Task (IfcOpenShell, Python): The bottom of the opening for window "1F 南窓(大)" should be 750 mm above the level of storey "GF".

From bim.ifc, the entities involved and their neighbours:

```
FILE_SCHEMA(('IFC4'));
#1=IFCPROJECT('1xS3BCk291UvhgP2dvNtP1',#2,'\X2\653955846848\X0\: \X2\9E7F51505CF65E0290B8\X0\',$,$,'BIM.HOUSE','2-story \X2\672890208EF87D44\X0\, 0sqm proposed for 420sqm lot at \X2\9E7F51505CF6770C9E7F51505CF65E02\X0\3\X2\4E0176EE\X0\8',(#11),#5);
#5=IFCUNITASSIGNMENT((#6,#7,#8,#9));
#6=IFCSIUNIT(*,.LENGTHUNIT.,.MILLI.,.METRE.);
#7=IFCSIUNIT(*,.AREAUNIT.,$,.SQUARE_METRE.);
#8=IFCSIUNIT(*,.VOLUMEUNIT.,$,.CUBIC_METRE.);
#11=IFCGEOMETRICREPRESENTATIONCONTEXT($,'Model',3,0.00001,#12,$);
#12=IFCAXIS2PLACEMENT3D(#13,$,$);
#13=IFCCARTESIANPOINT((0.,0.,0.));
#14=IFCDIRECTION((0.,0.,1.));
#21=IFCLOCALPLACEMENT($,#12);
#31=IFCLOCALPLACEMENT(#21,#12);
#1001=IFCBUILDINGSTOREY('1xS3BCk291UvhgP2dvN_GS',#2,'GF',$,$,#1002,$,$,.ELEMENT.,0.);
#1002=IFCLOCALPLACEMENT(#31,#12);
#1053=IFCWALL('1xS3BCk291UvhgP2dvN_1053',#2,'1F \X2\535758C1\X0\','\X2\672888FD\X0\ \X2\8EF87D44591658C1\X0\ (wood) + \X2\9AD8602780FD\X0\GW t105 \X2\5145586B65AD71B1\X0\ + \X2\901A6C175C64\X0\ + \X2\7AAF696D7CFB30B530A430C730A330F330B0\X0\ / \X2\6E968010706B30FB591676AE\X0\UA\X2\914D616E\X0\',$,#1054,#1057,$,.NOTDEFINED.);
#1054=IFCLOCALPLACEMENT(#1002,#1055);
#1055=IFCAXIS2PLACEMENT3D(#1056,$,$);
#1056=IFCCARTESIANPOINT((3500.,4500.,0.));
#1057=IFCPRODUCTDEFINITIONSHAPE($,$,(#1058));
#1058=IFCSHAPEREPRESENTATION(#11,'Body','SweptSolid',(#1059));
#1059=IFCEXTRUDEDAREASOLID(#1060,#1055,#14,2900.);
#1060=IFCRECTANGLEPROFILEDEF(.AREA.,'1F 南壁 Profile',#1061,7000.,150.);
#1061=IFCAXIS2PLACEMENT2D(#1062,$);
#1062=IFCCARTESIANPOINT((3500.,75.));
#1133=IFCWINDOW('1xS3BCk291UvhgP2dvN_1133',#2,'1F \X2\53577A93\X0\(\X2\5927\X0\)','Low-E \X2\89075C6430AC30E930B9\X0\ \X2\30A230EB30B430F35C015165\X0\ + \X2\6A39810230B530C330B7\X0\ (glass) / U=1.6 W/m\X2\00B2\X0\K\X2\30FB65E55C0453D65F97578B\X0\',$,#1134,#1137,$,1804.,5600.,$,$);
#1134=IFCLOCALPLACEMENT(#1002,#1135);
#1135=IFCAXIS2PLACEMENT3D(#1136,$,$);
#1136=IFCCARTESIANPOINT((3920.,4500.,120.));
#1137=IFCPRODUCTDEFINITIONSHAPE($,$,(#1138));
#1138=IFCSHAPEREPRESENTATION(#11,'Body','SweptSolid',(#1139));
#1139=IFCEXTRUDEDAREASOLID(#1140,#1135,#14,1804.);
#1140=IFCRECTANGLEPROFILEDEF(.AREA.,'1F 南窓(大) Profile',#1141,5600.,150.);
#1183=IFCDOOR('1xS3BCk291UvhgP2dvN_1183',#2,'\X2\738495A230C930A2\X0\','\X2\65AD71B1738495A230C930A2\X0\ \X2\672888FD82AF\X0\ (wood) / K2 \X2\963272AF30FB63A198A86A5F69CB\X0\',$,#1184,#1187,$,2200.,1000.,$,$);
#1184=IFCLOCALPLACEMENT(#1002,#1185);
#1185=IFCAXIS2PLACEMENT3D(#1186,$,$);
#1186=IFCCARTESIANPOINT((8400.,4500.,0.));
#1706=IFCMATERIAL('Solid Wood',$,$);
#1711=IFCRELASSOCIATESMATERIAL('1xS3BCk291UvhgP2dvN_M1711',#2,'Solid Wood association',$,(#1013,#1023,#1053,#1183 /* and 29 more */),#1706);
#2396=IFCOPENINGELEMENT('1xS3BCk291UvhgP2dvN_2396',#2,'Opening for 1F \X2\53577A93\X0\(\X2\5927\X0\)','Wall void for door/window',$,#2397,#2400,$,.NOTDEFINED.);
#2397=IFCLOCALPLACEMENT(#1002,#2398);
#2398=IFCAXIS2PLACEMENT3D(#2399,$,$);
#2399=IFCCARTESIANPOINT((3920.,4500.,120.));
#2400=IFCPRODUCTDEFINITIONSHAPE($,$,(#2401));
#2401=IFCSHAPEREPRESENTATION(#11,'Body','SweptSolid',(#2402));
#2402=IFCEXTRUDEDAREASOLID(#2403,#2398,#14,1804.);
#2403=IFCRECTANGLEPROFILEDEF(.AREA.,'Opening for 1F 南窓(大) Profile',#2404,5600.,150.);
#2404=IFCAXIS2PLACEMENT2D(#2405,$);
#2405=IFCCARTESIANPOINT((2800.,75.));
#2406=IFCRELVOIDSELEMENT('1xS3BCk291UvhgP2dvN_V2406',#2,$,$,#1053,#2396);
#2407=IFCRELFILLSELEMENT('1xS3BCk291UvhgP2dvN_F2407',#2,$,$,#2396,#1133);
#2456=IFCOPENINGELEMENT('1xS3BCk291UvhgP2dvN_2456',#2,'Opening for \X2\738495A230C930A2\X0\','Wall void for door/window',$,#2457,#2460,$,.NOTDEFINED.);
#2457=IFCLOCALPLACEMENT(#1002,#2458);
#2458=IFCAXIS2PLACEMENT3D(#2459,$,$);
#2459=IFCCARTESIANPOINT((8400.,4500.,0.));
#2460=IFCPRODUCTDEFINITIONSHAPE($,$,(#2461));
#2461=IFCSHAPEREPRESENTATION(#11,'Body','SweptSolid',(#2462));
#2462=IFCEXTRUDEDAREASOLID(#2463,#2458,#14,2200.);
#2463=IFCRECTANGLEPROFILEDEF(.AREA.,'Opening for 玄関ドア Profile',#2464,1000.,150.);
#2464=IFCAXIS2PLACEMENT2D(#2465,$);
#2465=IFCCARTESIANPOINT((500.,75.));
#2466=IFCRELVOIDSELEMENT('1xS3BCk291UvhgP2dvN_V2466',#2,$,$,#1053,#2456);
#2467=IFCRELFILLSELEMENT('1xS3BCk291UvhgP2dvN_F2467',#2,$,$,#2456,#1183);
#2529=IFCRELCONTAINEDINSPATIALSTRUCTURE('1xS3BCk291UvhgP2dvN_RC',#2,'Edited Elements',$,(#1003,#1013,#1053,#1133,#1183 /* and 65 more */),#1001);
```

```python
import numpy as np
import ifcopenshell
import ifcopenshell.api.geometry
import ifcopenshell.geom
import ifcopenshell.util.element
import ifcopenshell.util.placement
import ifcopenshell.util.shape
import ifcopenshell.util.unit

model = ifcopenshell.open("bim.ifc")
unit_scale = ifcopenshell.util.unit.calculate_unit_scale(model)

window = model.by_id(1133)
opening = window.FillsVoids[0].RelatingOpeningElement
storey = ifcopenshell.util.element.get_container(window, ifc_class="IfcBuildingStorey")
level = ifcopenshell.util.placement.get_local_placement(storey.ObjectPlacement)[2, 3]

# The opening's origin need not be at the sill, so measure its lowest point.
shape = ifcopenshell.geom.create_shape(ifcopenshell.geom.settings(), opening)
bottom = ifcopenshell.util.shape.get_shape_bottom_elevation(shape, shape.geometry) / unit_scale
dz = level + 0.75 / unit_scale - bottom

shift = np.array([0.0, 0.0, dz])
# The window is not placed relative to its opening, so move both.
for product in (opening, window):
    matrix = ifcopenshell.util.placement.get_local_placement(product.ObjectPlacement)
    matrix[:3, 3] += shift
    ifcopenshell.api.geometry.edit_object_placement(model, product=product, matrix=matrix, is_si=False)

print(f"moved by {dz * unit_scale:+.3f} m")

model.write("bim_rev.ifc")
```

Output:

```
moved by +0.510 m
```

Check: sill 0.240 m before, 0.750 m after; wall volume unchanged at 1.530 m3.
